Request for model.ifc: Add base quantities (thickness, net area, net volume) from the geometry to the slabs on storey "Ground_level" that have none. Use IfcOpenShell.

First a look at what the model holds.

```python
import ifcopenshell
import ifcopenshell.util.element
import ifcopenshell.util.unit

model = ifcopenshell.open("model.ifc")
print(model.schema)
for unit_type in ("LENGTHUNIT", "AREAUNIT", "VOLUMEUNIT"):
    print(unit_type, ifcopenshell.util.unit.calculate_unit_scale(model, unit_type))
storey = next(s for s in model.by_type("IfcBuildingStorey") if s.Name == "Ground_level")
slabs = [e for e in ifcopenshell.util.element.get_decomposition(storey) if e.is_a("IfcSlab")]
for e in sorted(slabs, key=lambda e: e.id()):
    print(e.id(), e.is_a(), e.Name, list(ifcopenshell.util.element.get_psets(e, qtos_only=True)), sep=" | ")
```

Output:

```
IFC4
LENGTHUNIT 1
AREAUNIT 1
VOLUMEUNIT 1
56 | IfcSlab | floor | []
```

```python
import ifcopenshell
import ifcopenshell.api.pset
import ifcopenshell.geom
import ifcopenshell.util.element
import ifcopenshell.util.shape
import ifcopenshell.util.unit

model = ifcopenshell.open("model.ifc")
unit_scale = ifcopenshell.util.unit.calculate_unit_scale(model)
area_scale = ifcopenshell.util.unit.calculate_unit_scale(model, "AREAUNIT")
volume_scale = ifcopenshell.util.unit.calculate_unit_scale(model, "VOLUMEUNIT")
settings = ifcopenshell.geom.settings()

storey = next(s for s in model.by_type("IfcBuildingStorey") if s.Name == "Ground_level")
slabs = [e for e in ifcopenshell.util.element.get_decomposition(storey) if e.is_a("IfcSlab")]

for e in sorted(slabs, key=lambda e: e.id()):
    if ifcopenshell.util.element.get_psets(e, qtos_only=True, should_inherit=False):
        continue
    # Geometry comes back in metres, in the element's own axes.
    shape = ifcopenshell.geom.create_shape(settings, e)
    values = {
        "Width": ifcopenshell.util.shape.get_z(shape.geometry) / unit_scale,
        "NetArea": ifcopenshell.util.shape.get_footprint_area(shape.geometry) / area_scale,
        "NetVolume": ifcopenshell.util.shape.get_volume(shape.geometry) / volume_scale,
    }
    qto = ifcopenshell.api.pset.add_qto(model, product=e, name="Qto_SlabBaseQuantities")
    ifcopenshell.api.pset.edit_qto(model, qto=qto, properties=values)
    print(e.id(), {k: round(v, 3) for k, v in values.items()})

model.write("model-out.ifc")
```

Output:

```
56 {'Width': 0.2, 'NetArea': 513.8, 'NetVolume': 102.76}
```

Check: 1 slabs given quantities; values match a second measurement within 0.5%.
